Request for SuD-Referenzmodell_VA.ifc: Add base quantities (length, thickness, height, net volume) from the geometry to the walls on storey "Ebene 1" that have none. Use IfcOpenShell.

First a look at what the model holds.

```python
import ifcopenshell
import ifcopenshell.util.element
import ifcopenshell.util.unit

model = ifcopenshell.open("SuD-Referenzmodell_VA.ifc")
print(model.schema)
for unit_type in ("LENGTHUNIT", "AREAUNIT", "VOLUMEUNIT"):
    print(unit_type, ifcopenshell.util.unit.calculate_unit_scale(model, unit_type))
storey = next(s for s in model.by_type("IfcBuildingStorey") if s.Name == "Ebene 1")
walls = [e for e in ifcopenshell.util.element.get_decomposition(storey) if e.is_a("IfcWall")]
for e in sorted(walls, key=lambda e: e.id()):
    print(e.id(), e.is_a(), e.Name, list(ifcopenshell.util.element.get_psets(e, qtos_only=True)), sep=" | ")
```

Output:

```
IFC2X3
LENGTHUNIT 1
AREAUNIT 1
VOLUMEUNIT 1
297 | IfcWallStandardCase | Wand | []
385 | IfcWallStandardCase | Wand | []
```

```python
import ifcopenshell
import ifcopenshell.api.pset
import ifcopenshell.geom
import ifcopenshell.util.element
import ifcopenshell.util.shape
import ifcopenshell.util.unit

model = ifcopenshell.open("SuD-Referenzmodell_VA.ifc")
unit_scale = ifcopenshell.util.unit.calculate_unit_scale(model)
volume_scale = ifcopenshell.util.unit.calculate_unit_scale(model, "VOLUMEUNIT")
settings = ifcopenshell.geom.settings()

storey = next(s for s in model.by_type("IfcBuildingStorey") if s.Name == "Ebene 1")
walls = [e for e in ifcopenshell.util.element.get_decomposition(storey) if e.is_a("IfcWall")]

for e in sorted(walls, key=lambda e: e.id()):
    if ifcopenshell.util.element.get_psets(e, qtos_only=True, should_inherit=False):
        continue
    # Geometry comes back in metres, in the element's own axes.
    shape = ifcopenshell.geom.create_shape(settings, e)
    values = {
        "Length": ifcopenshell.util.shape.get_x(shape.geometry) / unit_scale,
        "Width": ifcopenshell.util.shape.get_y(shape.geometry) / unit_scale,
        "Height": ifcopenshell.util.shape.get_z(shape.geometry) / unit_scale,
        "NetVolume": ifcopenshell.util.shape.get_volume(shape.geometry) / volume_scale,
    }
    qto = ifcopenshell.api.pset.add_qto(model, product=e, name="BaseQuantities")
    ifcopenshell.api.pset.edit_qto(model, qto=qto, properties=values)
    print(e.id(), {k: round(v, 3) for k, v in values.items()})

model.write("SuD-Referenzmodell_VA_updated.ifc")
```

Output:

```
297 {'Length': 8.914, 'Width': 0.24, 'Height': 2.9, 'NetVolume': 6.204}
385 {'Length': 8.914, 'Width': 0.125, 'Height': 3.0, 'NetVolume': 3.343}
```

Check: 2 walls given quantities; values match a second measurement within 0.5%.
